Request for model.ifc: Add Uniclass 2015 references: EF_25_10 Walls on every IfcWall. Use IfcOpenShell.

First a look at what the model holds.

```python
import ifcopenshell

model = ifcopenshell.open("model.ifc")
print(model.schema)
print("classifications:", [c.Name for c in model.by_type("IfcClassification")])
for ifc_class in ("IfcDoor", "IfcRoof", "IfcStair", "IfcWall", "IfcWindow"):
    print(ifc_class, len(model.by_type(ifc_class)))
```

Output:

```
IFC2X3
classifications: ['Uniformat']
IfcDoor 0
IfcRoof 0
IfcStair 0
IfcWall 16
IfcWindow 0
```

```python
import ifcopenshell
import ifcopenshell.api.classification

model = ifcopenshell.open("model.ifc")

# IFC2X3 requires Source and Edition and has no link from the project to the system.
system = model.create_entity("IfcClassification", Source="NBS", Edition="2015", Name="Uniclass 2015")

codes = {
    "IfcWall": ("EF_25_10", "Walls"),
}
for ifc_class, (code, name) in codes.items():
    products = model.by_type(ifc_class)
    ifcopenshell.api.classification.add_reference(
        model, products=products, classification=system, identification=code, name=name
    )
    print(code, len(products))

model.write("model_updated.ifc")
```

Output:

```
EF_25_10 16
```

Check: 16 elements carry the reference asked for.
